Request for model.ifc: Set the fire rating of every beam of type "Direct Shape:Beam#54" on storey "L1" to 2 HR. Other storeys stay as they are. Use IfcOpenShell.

First a look at what the model holds.

```python
import ifcopenshell
import ifcopenshell.util.element

model = ifcopenshell.open("model.ifc")
print(model.schema)
storey = next(s for s in model.by_type("IfcBuildingStorey") if s.Name == "L1")
beams = [e for e in ifcopenshell.util.element.get_decomposition(storey) if e.is_a("IfcBeam")]
seen = {}
for e in beams:
    element_type = ifcopenshell.util.element.get_type(e)
    key = (element_type.Name if element_type != e and element_type else None, ifcopenshell.util.element.get_pset(e, "Pset_BeamCommon", "FireRating"))
    seen[key] = seen.get(key, 0) + 1
for (name, value), count in sorted(seen.items(), key=str):
    print(count, "x", name, "|", value)
```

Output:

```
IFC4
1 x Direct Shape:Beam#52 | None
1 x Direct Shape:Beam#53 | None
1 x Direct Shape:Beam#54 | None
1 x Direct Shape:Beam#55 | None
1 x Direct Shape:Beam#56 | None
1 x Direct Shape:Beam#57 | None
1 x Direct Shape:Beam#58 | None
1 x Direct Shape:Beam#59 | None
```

```python
import ifcopenshell
import ifcopenshell.api.pset
import ifcopenshell.util.element

model = ifcopenshell.open("model.ifc")

storey = next(s for s in model.by_type("IfcBuildingStorey") if s.Name == "L1")
beams = [e for e in ifcopenshell.util.element.get_decomposition(storey) if e.is_a("IfcBeam")]

count = 0
for e in beams:
    element_type = ifcopenshell.util.element.get_type(e)
    if element_type in (None, e) or element_type.Name != "Direct Shape:Beam#54":
        continue
    # add_pset returns the element's existing set when there is one.
    pset = ifcopenshell.api.pset.add_pset(model, product=e, name="Pset_BeamCommon")
    ifcopenshell.api.pset.edit_pset(model, pset=pset, properties={"FireRating": "2 HR"})
    count += 1

print(count, "beams updated")

model.write("model_rev.ifc")
```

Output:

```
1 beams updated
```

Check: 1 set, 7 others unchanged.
